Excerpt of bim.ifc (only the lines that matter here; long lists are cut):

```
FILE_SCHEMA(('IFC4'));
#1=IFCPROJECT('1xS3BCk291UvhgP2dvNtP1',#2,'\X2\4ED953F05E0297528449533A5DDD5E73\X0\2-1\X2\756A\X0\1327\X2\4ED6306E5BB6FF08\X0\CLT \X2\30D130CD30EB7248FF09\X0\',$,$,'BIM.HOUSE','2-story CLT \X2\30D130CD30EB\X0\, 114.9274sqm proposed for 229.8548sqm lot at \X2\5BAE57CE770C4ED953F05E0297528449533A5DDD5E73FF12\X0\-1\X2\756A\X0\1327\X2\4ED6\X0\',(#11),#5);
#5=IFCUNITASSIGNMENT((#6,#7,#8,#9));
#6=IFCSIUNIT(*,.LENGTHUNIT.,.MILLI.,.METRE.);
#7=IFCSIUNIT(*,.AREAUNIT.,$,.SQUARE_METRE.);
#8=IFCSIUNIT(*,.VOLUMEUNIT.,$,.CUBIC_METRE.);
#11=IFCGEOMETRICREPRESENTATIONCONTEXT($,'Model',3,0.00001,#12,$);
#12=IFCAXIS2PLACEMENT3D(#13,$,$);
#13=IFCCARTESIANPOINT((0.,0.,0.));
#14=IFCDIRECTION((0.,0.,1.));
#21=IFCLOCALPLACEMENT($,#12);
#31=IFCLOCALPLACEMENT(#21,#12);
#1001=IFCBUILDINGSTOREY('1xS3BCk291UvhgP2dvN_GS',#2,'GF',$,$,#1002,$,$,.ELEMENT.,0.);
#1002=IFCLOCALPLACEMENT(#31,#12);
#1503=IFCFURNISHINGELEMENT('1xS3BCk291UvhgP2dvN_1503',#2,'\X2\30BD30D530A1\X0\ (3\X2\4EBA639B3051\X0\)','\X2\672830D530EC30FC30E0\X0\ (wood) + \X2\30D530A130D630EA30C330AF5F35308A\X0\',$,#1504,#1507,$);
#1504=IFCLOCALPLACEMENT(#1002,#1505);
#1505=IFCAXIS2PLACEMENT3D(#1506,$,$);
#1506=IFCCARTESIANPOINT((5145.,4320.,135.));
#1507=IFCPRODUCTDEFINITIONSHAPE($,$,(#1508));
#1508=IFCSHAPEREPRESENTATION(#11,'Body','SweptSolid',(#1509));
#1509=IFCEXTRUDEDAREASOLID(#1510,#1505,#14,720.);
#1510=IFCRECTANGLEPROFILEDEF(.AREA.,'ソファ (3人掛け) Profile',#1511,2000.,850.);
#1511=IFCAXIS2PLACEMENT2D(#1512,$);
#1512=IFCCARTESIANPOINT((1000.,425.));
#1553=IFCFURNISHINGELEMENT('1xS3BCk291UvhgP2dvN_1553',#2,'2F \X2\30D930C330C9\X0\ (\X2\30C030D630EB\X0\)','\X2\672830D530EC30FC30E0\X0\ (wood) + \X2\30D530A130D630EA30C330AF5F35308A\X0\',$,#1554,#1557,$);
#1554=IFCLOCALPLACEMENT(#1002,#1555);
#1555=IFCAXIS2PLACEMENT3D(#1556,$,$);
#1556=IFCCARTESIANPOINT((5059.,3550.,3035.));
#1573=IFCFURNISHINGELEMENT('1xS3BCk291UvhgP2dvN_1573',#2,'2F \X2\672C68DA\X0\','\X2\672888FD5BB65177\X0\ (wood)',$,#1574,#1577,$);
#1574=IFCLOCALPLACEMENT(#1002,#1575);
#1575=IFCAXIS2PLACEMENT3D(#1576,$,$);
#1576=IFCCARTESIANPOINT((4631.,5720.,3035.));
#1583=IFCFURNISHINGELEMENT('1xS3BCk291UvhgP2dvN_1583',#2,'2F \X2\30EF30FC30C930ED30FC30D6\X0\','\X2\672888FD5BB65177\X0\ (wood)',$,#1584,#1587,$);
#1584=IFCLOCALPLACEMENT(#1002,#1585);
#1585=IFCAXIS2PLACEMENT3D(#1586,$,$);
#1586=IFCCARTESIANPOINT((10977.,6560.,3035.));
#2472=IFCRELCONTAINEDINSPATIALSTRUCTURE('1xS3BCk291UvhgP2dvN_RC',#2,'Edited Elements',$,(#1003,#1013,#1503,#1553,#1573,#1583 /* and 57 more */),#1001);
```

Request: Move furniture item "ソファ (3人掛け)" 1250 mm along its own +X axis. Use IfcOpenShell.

```python
import ifcopenshell
import ifcopenshell.api.geometry
import ifcopenshell.util.placement

model = ifcopenshell.open("bim.ifc")

item = model.by_id(1503)
matrix = ifcopenshell.util.placement.get_local_placement(item.ObjectPlacement)
matrix[:3, 3] += matrix[:3, 0] * 1250.0
ifcopenshell.api.geometry.edit_object_placement(model, product=item, matrix=matrix, is_si=False)

print(ifcopenshell.util.placement.get_local_placement(item.ObjectPlacement).round(3) + 0.0)

model.write("bim-out.ifc")
```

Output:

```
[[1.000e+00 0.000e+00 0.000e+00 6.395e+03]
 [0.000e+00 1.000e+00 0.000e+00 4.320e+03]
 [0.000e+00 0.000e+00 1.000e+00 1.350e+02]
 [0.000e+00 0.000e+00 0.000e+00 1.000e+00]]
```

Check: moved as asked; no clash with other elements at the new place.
